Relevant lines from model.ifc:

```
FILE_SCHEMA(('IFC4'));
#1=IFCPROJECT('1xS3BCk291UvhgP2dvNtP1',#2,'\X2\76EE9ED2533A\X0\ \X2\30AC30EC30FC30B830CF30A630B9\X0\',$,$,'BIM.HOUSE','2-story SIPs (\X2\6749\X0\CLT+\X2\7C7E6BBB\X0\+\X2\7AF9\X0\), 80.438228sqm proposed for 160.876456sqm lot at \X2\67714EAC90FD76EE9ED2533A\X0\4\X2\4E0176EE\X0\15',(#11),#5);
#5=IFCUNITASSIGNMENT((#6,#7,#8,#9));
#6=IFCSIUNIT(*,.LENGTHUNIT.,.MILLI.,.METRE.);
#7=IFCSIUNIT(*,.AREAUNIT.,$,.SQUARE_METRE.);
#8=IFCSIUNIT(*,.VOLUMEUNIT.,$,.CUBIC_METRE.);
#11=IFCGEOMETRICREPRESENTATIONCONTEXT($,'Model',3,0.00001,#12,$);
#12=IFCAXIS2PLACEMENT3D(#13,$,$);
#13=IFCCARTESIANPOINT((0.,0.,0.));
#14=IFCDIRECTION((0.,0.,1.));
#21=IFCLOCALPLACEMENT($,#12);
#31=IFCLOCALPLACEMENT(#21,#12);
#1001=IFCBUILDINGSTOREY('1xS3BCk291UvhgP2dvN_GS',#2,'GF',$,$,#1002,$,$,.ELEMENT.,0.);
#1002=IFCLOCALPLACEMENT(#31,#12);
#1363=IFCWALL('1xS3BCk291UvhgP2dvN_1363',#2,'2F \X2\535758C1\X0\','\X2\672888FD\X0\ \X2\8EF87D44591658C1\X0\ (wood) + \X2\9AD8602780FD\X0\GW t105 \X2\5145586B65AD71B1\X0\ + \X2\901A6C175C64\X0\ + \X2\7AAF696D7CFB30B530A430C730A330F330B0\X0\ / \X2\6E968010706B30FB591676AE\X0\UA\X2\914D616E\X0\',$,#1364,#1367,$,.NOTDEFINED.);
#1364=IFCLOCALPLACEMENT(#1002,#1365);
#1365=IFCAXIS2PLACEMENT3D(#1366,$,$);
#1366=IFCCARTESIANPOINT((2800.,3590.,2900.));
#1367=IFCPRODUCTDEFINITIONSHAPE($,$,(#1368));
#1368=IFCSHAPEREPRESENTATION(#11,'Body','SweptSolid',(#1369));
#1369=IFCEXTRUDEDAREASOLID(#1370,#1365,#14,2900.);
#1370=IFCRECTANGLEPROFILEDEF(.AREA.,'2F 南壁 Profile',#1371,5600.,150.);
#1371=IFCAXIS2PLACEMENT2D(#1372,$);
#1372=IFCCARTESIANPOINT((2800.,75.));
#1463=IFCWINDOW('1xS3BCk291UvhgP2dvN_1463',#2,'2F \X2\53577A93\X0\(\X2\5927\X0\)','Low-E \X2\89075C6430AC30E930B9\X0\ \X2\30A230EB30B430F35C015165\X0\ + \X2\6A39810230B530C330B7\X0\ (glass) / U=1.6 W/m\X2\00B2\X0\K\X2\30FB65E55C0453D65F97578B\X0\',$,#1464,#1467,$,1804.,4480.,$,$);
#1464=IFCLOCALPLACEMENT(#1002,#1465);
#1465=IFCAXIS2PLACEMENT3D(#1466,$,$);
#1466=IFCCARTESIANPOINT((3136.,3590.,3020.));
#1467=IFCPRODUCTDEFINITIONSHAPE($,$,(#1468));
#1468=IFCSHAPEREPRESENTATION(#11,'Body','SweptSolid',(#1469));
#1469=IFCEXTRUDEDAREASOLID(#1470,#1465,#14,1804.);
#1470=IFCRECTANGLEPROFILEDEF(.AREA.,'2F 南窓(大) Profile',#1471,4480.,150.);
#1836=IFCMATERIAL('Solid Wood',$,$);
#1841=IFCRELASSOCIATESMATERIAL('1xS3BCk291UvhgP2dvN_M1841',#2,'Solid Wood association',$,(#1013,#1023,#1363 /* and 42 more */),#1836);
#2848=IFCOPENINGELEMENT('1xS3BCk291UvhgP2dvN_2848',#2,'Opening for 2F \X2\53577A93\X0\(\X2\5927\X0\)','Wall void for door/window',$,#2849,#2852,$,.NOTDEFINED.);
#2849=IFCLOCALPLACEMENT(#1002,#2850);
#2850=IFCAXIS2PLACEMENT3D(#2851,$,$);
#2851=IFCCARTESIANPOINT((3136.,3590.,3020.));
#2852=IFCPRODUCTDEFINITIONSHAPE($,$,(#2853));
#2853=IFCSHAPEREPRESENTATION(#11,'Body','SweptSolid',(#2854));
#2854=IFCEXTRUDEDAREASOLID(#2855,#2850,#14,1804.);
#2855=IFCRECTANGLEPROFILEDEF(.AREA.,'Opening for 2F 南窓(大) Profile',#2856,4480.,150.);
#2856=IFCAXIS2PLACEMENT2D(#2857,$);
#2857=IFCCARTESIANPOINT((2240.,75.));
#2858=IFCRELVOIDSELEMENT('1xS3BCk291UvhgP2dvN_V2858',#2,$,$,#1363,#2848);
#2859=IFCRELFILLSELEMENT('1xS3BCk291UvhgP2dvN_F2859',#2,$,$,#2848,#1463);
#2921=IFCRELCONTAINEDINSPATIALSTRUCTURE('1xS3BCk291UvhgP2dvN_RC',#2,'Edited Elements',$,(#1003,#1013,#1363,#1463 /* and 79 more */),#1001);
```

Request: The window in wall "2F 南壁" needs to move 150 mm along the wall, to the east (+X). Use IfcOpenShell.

```python
import ifcopenshell
import ifcopenshell.api.geometry
import ifcopenshell.util.placement

model = ifcopenshell.open("model.ifc")

window = model.by_id(1463)
opening = window.FillsVoids[0].RelatingOpeningElement
wall = opening.VoidsElements[0].RelatingBuildingElement

wall_matrix = ifcopenshell.util.placement.get_local_placement(wall.ObjectPlacement)
shift = wall_matrix[:3, 0] * 150.0
before = ifcopenshell.util.placement.get_local_placement(window.ObjectPlacement)[:3, 3].copy()

# The window is not placed relative to its opening, so move both.
for product in (opening, window):
    matrix = ifcopenshell.util.placement.get_local_placement(product.ObjectPlacement)
    matrix[:3, 3] += shift
    ifcopenshell.api.geometry.edit_object_placement(model, product=product, matrix=matrix, is_si=False)

after = ifcopenshell.util.placement.get_local_placement(window.ObjectPlacement)[:3, 3]
print("window moved by", (after - before).round(3) + 0.0)

model.write("model_edited.ifc")
```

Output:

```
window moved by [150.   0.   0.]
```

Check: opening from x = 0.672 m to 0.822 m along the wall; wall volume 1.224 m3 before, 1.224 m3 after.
